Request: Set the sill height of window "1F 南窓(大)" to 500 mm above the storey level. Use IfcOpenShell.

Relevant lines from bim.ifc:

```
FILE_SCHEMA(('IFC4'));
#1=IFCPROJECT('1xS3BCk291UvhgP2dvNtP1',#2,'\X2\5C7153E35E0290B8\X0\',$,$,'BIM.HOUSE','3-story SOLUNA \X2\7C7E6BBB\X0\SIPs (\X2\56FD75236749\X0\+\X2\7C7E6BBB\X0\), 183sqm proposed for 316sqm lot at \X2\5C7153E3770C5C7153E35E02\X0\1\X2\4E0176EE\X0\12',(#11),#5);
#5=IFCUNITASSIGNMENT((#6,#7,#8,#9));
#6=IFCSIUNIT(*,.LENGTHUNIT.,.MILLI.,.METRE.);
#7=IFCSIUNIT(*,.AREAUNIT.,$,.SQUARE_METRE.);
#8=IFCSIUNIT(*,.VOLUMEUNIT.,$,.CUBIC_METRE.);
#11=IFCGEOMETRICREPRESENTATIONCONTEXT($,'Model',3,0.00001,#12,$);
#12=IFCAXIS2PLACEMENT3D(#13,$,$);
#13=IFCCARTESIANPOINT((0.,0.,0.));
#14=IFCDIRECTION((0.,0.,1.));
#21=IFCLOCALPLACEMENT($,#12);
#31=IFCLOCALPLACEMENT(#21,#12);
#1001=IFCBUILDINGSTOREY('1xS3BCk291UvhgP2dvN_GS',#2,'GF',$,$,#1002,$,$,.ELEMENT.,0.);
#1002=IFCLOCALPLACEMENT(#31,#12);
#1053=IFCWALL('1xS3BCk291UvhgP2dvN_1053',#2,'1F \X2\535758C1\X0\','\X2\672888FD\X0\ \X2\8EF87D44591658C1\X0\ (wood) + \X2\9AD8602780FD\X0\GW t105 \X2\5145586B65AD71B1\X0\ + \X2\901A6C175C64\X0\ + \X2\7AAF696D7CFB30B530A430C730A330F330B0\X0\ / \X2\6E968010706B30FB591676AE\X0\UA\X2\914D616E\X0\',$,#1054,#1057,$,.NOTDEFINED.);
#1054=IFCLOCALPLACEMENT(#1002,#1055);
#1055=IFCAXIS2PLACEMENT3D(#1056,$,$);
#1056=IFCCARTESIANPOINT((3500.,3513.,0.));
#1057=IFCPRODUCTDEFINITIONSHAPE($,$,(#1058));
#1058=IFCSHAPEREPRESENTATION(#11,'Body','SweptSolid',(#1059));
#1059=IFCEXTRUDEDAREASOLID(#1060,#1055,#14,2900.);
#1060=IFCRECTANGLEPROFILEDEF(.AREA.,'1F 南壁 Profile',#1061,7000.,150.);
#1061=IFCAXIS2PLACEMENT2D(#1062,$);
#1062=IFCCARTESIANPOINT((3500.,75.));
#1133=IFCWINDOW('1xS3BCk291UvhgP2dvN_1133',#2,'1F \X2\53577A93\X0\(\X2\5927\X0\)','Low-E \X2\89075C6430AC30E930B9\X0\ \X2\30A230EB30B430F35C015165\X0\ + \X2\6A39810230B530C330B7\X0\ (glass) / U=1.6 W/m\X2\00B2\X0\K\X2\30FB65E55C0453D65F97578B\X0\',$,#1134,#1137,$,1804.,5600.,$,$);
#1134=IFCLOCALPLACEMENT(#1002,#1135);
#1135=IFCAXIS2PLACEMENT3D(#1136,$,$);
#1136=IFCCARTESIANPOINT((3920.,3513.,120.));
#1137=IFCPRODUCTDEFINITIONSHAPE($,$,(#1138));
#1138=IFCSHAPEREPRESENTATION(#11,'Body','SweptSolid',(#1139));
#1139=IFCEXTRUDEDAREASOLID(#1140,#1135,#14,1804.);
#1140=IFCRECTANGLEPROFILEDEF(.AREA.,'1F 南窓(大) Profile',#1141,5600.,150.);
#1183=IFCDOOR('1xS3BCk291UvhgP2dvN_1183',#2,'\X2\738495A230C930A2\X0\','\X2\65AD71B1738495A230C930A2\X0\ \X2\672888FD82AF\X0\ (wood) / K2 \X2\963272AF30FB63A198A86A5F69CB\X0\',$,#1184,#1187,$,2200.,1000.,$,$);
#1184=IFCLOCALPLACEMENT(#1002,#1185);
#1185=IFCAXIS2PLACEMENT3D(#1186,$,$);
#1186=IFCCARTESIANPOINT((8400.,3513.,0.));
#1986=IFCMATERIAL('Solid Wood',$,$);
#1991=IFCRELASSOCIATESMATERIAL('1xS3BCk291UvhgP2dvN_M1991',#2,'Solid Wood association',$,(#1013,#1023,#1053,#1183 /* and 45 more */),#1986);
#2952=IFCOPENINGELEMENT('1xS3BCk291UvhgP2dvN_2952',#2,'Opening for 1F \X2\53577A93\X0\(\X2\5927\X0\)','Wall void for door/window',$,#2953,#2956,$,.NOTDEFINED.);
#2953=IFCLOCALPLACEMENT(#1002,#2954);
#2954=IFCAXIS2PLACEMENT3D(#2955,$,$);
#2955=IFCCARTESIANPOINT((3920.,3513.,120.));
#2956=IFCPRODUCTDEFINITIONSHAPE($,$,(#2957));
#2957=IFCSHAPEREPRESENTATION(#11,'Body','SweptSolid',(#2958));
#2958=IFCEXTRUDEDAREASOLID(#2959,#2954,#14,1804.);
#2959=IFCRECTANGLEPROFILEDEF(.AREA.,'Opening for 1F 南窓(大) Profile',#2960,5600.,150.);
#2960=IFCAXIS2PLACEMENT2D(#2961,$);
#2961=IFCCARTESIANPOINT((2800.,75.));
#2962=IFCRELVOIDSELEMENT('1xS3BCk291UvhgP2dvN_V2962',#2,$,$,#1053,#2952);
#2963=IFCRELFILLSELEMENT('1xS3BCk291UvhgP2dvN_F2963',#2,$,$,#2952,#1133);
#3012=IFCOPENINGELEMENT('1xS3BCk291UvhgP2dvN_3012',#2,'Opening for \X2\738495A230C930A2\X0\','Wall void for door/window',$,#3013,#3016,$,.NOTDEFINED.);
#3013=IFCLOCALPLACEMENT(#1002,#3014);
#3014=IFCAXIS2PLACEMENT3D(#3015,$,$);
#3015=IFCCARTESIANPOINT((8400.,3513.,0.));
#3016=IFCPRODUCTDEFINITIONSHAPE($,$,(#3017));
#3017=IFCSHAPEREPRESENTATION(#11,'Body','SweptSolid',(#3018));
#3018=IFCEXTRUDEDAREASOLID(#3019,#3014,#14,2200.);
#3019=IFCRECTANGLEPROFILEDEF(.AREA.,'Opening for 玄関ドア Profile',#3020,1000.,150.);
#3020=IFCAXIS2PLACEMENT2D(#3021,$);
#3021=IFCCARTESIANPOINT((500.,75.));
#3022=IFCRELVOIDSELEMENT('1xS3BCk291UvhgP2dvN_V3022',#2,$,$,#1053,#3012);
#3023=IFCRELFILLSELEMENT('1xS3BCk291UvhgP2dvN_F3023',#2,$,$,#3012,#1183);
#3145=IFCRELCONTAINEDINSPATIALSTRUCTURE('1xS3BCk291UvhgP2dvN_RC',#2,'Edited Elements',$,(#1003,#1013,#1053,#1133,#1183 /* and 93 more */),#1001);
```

```python
import numpy as np
import ifcopenshell
import ifcopenshell.api.geometry
import ifcopenshell.geom
import ifcopenshell.util.element
import ifcopenshell.util.placement
import ifcopenshell.util.shape
import ifcopenshell.util.unit

model = ifcopenshell.open("bim.ifc")
unit_scale = ifcopenshell.util.unit.calculate_unit_scale(model)

window = model.by_guid("1xS3BCk291UvhgP2dvN_1133")
opening = window.FillsVoids[0].RelatingOpeningElement
storey = ifcopenshell.util.element.get_container(window, ifc_class="IfcBuildingStorey")
level = ifcopenshell.util.placement.get_local_placement(storey.ObjectPlacement)[2, 3]

# The opening's origin need not be at the sill, so measure its lowest point.
shape = ifcopenshell.geom.create_shape(ifcopenshell.geom.settings(), opening)
bottom = ifcopenshell.util.shape.get_shape_bottom_elevation(shape, shape.geometry) / unit_scale
dz = level + 0.5 / unit_scale - bottom

shift = np.array([0.0, 0.0, dz])
# The window is not placed relative to its opening, so move both.
for product in (opening, window):
    matrix = ifcopenshell.util.placement.get_local_placement(product.ObjectPlacement)
    matrix[:3, 3] += shift
    ifcopenshell.api.geometry.edit_object_placement(model, product=product, matrix=matrix, is_si=False)

print(f"moved by {dz * unit_scale:+.3f} m")

model.write("bim_v2.ifc")
```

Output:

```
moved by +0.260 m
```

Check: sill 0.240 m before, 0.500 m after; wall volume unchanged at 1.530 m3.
